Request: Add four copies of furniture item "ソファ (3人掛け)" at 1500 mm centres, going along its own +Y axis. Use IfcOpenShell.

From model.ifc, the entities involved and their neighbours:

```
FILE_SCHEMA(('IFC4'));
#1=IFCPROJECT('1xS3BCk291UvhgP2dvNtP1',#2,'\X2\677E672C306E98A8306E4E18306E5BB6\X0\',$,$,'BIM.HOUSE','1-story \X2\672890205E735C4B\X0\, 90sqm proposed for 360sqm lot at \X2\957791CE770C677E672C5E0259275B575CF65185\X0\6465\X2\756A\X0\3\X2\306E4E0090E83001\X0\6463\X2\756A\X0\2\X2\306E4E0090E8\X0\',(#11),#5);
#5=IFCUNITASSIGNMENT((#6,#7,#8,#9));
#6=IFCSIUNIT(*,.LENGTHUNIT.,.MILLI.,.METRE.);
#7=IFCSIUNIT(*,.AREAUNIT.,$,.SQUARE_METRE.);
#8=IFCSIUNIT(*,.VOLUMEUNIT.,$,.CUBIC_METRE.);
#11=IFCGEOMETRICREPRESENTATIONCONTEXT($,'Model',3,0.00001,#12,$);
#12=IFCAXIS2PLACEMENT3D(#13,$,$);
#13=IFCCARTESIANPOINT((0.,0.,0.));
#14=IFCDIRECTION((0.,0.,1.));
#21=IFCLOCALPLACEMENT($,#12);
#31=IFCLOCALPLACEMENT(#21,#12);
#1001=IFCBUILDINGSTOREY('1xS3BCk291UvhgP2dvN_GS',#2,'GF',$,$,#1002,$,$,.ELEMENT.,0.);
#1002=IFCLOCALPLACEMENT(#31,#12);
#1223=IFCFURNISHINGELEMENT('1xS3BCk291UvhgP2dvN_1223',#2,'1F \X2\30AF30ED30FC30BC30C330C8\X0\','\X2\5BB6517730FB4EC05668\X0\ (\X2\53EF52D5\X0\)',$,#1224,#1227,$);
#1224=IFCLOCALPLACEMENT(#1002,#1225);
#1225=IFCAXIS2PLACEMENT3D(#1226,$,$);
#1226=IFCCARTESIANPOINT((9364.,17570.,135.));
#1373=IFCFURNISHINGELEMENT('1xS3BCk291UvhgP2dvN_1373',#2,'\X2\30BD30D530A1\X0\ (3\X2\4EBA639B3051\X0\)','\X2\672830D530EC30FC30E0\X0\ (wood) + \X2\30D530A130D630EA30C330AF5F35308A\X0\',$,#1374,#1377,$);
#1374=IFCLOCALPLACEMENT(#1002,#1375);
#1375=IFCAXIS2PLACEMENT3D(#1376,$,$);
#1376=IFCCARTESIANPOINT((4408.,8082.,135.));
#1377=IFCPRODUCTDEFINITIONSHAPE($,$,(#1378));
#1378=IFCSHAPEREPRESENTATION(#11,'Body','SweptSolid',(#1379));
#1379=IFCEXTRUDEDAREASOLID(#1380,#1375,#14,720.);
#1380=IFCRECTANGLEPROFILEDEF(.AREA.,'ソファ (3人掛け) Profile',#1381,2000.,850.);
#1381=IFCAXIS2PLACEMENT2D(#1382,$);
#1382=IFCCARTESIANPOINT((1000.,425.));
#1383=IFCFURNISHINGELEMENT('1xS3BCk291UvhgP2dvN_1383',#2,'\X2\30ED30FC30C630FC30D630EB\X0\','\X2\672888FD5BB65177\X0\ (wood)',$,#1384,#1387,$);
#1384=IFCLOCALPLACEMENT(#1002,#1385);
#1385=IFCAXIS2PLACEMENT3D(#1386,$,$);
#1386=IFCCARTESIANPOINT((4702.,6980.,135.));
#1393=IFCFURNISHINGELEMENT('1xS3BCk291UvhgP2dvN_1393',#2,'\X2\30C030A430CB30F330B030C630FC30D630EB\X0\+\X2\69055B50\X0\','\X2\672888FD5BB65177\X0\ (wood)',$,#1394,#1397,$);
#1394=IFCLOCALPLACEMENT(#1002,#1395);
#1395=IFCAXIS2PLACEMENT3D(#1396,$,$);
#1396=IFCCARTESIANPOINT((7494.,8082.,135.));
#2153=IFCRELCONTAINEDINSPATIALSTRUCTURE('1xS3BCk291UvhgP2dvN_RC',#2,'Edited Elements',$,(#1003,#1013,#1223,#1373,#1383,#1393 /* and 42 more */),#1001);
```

```python
import ifcopenshell
import ifcopenshell.api.geometry
import ifcopenshell.api.root
import ifcopenshell.util.element
import ifcopenshell.util.placement

model = ifcopenshell.open("model.ifc")


def reuse_history(source, copy):
    """copy_class also copies each property set's owner history, people and application; keep the originals."""
    for rel in copy.IsDefinedBy:
        if rel.is_a("IfcRelDefinesByProperties") and (history := rel.RelatingPropertyDefinition.OwnerHistory):
            rel.RelatingPropertyDefinition.OwnerHistory = source.OwnerHistory
            ifcopenshell.util.element.remove_deep2(model, history)


source = model.by_guid("1xS3BCk291UvhgP2dvN_1373")
base = ifcopenshell.util.placement.get_local_placement(source.ObjectPlacement)
step = base[:3, 1] * 1500.0

for i in range(1, 5):
    copy = ifcopenshell.api.root.copy_class(model, product=source)
    copy.Representation = ifcopenshell.util.element.copy_deep(
        model, source.Representation, exclude=["IfcGeometricRepresentationContext", "IfcRepresentationMap"]
    )
    reuse_history(source, copy)
    matrix = base.copy()
    matrix[:3, 3] += i * step
    print("added at", matrix[:3, 3].round(3) + 0.0)
    ifcopenshell.api.geometry.edit_object_placement(model, product=copy, matrix=matrix, is_si=False)

model.write("model-out.ifc")
```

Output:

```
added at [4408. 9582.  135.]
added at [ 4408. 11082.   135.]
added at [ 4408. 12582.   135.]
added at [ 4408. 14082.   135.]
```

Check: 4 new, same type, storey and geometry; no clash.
